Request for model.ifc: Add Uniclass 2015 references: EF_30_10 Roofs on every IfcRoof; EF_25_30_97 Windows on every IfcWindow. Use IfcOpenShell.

First a look at what the model holds.

```python
import ifcopenshell

model = ifcopenshell.open("model.ifc")
print(model.schema)
print("classifications:", [c.Name for c in model.by_type("IfcClassification")])
for ifc_class in ("IfcDoor", "IfcRoof", "IfcStair", "IfcWall", "IfcWindow"):
    print(ifc_class, len(model.by_type(ifc_class)))
```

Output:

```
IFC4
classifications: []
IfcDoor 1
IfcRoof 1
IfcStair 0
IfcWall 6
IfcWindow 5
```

```python
import ifcopenshell
import ifcopenshell.api.classification

model = ifcopenshell.open("model.ifc")

system = ifcopenshell.api.classification.add_classification(model, classification="Uniclass 2015")

codes = {
    "IfcRoof": ("EF_30_10", "Roofs"),
    "IfcWindow": ("EF_25_30_97", "Windows"),
}
for ifc_class, (code, name) in codes.items():
    products = model.by_type(ifc_class)
    ifcopenshell.api.classification.add_reference(
        model, products=products, classification=system, identification=code, name=name
    )
    print(code, len(products))

model.write("model_v2.ifc")
```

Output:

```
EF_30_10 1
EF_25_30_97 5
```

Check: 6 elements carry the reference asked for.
